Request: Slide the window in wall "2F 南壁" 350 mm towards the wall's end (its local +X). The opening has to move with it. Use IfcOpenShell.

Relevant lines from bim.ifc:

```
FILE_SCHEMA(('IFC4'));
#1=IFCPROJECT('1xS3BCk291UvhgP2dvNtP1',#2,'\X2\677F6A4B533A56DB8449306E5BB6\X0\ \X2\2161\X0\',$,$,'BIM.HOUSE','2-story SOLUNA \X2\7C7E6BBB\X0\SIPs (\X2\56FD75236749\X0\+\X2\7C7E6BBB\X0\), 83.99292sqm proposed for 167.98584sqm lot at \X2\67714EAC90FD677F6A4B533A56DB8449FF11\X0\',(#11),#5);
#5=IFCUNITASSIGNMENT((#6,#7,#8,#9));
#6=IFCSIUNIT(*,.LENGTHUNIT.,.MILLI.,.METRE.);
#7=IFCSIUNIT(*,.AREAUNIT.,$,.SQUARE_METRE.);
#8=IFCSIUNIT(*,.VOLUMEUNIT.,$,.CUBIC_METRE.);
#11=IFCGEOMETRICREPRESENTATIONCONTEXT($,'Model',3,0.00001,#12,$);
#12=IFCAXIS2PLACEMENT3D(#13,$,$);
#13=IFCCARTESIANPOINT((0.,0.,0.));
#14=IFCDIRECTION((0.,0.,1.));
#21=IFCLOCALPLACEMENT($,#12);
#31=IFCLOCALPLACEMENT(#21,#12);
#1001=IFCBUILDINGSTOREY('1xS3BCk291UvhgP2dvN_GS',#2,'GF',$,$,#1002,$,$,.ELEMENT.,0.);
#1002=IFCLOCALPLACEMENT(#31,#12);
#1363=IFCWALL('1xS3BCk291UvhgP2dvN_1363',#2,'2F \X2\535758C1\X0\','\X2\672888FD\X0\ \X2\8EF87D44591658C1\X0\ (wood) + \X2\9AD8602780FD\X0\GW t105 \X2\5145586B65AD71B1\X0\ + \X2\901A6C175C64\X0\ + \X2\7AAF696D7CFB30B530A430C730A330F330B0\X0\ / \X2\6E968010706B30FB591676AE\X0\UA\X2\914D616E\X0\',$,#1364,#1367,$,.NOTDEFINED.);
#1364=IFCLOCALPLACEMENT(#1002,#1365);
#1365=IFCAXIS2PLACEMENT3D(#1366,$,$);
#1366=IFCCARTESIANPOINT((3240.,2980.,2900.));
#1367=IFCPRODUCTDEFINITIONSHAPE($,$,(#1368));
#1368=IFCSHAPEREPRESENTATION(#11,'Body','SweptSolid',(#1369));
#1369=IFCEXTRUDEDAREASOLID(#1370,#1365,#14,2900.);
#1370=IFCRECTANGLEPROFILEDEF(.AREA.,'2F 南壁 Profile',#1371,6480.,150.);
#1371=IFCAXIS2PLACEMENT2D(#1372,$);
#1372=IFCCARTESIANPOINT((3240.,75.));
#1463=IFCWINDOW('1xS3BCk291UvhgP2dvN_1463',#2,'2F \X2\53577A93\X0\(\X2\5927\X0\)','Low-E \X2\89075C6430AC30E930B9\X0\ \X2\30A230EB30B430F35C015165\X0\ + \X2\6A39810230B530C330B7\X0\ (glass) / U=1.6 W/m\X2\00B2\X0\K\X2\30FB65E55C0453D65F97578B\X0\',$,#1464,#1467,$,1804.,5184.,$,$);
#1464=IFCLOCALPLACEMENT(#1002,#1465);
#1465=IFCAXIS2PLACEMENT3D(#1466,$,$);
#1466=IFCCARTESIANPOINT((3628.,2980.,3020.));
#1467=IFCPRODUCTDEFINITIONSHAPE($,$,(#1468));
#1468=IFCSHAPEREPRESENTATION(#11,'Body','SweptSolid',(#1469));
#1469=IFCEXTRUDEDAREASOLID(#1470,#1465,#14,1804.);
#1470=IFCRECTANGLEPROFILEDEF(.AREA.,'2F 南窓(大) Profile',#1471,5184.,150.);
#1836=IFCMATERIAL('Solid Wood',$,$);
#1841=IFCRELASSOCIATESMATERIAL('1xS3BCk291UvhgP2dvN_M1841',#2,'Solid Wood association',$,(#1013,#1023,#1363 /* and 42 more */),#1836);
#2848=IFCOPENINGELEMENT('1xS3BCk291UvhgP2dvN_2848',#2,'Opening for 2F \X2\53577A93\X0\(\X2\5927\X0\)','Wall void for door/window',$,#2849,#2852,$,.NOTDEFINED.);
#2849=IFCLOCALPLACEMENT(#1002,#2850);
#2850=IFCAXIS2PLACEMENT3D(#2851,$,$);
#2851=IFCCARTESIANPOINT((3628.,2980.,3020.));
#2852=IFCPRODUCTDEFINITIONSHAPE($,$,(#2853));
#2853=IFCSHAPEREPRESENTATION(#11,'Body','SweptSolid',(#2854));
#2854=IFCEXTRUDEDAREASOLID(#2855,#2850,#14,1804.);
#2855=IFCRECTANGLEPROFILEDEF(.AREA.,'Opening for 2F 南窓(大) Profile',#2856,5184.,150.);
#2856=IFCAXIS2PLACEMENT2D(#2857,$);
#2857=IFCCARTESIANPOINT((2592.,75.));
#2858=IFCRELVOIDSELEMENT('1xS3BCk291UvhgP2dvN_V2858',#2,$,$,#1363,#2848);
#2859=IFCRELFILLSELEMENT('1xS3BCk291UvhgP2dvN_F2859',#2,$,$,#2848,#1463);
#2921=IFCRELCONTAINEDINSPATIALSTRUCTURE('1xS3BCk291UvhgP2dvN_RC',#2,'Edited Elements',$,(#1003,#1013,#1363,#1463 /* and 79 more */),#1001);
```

```python
import ifcopenshell
import ifcopenshell.api.geometry
import ifcopenshell.util.placement
import ifcopenshell.util.unit

model = ifcopenshell.open("bim.ifc")
unit_scale = ifcopenshell.util.unit.calculate_unit_scale(model)

window = model.by_guid("1xS3BCk291UvhgP2dvN_1463")
opening = window.FillsVoids[0].RelatingOpeningElement
wall = opening.VoidsElements[0].RelatingBuildingElement

wall_matrix = ifcopenshell.util.placement.get_local_placement(wall.ObjectPlacement)
shift = wall_matrix[:3, 0] * 0.35 / unit_scale
before = ifcopenshell.util.placement.get_local_placement(window.ObjectPlacement)[:3, 3].copy()

# The window is not placed relative to its opening, so move both.
for product in (opening, window):
    matrix = ifcopenshell.util.placement.get_local_placement(product.ObjectPlacement)
    matrix[:3, 3] += shift
    ifcopenshell.api.geometry.edit_object_placement(model, product=product, matrix=matrix, is_si=False)

after = ifcopenshell.util.placement.get_local_placement(window.ObjectPlacement)[:3, 3]
print("window moved by", (after - before).round(3) + 0.0)

model.write("bim_rev.ifc")
```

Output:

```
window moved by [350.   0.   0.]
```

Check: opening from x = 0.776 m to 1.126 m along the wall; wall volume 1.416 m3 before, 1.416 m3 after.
